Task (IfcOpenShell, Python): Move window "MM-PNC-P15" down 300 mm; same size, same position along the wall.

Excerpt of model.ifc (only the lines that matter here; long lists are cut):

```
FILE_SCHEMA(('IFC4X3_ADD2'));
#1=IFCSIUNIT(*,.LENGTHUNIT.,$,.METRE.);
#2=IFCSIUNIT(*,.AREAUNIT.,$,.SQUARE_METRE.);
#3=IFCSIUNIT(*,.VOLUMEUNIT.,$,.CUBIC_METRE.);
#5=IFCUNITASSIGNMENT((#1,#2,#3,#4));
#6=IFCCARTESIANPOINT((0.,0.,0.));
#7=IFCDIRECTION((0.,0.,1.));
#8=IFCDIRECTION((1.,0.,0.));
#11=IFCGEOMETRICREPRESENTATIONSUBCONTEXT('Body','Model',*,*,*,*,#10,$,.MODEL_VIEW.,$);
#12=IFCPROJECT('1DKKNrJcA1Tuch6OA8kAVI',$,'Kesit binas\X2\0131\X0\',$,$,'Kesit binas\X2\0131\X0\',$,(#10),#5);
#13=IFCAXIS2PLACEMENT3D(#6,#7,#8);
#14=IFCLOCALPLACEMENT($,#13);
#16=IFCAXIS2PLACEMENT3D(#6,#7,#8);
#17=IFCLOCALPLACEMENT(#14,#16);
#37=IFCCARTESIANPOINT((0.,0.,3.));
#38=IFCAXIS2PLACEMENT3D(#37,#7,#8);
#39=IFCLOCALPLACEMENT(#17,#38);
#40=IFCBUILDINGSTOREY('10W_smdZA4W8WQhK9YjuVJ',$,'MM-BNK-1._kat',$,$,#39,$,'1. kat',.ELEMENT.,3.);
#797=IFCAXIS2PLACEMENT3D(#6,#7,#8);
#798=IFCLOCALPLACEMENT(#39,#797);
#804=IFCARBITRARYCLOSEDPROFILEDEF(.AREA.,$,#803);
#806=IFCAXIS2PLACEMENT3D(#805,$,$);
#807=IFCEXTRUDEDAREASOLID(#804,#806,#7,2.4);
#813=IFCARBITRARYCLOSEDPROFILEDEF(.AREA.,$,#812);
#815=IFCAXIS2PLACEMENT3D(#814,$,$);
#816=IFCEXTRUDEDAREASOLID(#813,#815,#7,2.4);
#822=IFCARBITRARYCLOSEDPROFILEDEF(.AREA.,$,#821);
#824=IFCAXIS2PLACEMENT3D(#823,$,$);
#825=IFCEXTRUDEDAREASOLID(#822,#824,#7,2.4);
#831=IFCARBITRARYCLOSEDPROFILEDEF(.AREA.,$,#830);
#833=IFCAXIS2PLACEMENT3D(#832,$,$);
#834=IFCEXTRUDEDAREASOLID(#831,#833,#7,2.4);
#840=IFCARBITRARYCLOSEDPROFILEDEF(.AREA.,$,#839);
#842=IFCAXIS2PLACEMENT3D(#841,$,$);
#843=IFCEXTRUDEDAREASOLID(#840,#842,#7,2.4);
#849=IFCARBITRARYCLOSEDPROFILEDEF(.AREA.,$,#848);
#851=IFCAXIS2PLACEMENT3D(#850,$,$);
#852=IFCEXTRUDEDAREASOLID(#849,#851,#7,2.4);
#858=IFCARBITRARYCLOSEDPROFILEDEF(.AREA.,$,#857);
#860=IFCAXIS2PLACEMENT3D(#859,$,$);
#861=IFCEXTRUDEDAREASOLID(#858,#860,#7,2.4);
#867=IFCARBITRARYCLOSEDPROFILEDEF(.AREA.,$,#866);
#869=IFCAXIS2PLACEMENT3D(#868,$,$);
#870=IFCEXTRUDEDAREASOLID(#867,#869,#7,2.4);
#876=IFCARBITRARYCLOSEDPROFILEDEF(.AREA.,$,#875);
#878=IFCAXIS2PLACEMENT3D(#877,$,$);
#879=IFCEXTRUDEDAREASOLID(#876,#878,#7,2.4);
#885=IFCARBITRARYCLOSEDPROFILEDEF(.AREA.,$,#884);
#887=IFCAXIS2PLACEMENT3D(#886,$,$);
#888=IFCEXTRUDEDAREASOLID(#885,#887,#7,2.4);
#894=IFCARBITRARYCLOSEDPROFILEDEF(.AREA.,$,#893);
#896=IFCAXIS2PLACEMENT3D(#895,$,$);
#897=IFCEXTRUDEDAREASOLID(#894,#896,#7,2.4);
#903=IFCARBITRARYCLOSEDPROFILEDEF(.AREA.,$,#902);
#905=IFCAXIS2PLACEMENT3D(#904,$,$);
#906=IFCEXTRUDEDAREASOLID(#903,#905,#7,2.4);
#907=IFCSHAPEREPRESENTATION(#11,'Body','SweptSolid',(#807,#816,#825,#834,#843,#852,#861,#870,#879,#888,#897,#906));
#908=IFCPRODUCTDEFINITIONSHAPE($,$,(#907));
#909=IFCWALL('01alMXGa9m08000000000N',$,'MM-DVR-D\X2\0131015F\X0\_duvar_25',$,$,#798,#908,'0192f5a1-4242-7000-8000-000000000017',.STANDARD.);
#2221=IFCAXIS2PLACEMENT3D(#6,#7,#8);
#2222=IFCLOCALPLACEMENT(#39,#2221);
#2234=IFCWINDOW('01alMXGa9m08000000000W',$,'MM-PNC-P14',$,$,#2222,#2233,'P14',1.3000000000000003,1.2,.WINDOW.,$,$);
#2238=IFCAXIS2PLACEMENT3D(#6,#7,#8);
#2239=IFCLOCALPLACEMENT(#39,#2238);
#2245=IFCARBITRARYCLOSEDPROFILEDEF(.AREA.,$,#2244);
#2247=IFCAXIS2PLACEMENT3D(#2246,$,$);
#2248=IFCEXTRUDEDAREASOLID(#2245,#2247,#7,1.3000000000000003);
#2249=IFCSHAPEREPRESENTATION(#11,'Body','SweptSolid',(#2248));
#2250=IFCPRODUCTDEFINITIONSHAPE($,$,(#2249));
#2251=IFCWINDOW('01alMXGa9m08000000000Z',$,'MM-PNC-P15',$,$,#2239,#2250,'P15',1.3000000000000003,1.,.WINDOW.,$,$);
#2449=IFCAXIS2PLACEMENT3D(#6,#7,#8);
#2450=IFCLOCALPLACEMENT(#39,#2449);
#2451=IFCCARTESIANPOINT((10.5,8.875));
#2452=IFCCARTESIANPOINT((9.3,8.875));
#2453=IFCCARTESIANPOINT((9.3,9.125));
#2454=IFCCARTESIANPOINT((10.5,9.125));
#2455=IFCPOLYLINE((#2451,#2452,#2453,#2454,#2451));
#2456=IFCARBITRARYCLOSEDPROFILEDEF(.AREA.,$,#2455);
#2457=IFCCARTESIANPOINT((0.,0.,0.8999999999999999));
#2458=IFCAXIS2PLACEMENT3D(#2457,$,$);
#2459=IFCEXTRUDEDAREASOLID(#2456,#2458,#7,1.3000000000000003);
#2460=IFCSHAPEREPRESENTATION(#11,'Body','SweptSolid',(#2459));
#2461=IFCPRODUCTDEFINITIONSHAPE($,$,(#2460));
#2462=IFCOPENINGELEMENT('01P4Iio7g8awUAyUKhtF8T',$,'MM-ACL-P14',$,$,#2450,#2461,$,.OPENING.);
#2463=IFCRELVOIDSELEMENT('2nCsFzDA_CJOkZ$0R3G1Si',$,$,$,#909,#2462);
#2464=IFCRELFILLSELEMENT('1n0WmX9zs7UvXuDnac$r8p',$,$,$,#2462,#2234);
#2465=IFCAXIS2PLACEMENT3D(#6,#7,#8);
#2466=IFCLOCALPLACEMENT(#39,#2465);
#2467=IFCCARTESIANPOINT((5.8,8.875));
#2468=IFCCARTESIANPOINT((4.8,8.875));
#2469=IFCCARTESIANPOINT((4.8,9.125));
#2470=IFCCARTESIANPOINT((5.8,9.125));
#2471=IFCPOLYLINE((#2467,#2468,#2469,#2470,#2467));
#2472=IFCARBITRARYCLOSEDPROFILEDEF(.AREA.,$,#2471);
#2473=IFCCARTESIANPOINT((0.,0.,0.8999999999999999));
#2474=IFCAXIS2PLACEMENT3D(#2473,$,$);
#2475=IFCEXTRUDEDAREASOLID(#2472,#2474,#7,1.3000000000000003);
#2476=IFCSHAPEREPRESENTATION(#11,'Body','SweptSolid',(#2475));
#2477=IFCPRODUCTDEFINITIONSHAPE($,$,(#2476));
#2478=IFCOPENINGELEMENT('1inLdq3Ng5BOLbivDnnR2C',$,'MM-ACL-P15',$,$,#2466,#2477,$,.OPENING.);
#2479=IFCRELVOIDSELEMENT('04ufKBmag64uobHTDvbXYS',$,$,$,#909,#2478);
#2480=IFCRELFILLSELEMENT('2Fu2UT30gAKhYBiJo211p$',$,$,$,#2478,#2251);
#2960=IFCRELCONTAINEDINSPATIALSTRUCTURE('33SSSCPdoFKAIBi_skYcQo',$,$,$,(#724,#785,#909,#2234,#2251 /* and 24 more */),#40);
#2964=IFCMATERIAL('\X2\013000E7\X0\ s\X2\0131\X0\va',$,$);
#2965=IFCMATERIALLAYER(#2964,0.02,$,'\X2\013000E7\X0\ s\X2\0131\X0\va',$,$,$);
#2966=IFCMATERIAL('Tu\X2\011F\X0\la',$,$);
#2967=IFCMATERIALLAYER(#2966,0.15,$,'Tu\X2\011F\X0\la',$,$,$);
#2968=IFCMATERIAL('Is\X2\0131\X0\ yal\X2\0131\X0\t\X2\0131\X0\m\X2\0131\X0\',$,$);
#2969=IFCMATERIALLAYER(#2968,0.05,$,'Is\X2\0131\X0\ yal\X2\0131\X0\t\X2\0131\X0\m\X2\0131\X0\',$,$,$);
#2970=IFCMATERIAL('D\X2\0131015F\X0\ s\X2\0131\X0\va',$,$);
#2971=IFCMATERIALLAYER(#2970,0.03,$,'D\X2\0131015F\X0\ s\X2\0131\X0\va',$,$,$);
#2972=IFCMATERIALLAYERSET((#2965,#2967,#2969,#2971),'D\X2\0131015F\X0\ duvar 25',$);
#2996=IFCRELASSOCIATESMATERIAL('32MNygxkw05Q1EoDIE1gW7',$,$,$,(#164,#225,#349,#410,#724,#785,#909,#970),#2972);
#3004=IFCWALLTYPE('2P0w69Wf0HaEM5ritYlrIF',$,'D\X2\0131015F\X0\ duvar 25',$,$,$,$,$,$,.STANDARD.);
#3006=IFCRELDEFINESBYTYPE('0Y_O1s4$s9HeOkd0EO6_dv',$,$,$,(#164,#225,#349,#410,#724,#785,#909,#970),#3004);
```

```python
import numpy as np
import ifcopenshell
import ifcopenshell.api.geometry
import ifcopenshell.util.placement
import ifcopenshell.util.unit

model = ifcopenshell.open("model.ifc")
unit_scale = ifcopenshell.util.unit.calculate_unit_scale(model)

window = model.by_guid("01alMXGa9m08000000000Z")
opening = window.FillsVoids[0].RelatingOpeningElement
dz = -0.3

shift = np.array([0.0, 0.0, dz])
# The window is not placed relative to its opening, so move both.
for product in (opening, window):
    matrix = ifcopenshell.util.placement.get_local_placement(product.ObjectPlacement)
    matrix[:3, 3] += shift
    ifcopenshell.api.geometry.edit_object_placement(model, product=product, matrix=matrix, is_si=False)

print(f"moved by {dz * unit_scale:+.3f} m")

model.write("model_v2.ifc")
```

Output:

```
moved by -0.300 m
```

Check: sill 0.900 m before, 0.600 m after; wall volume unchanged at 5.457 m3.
